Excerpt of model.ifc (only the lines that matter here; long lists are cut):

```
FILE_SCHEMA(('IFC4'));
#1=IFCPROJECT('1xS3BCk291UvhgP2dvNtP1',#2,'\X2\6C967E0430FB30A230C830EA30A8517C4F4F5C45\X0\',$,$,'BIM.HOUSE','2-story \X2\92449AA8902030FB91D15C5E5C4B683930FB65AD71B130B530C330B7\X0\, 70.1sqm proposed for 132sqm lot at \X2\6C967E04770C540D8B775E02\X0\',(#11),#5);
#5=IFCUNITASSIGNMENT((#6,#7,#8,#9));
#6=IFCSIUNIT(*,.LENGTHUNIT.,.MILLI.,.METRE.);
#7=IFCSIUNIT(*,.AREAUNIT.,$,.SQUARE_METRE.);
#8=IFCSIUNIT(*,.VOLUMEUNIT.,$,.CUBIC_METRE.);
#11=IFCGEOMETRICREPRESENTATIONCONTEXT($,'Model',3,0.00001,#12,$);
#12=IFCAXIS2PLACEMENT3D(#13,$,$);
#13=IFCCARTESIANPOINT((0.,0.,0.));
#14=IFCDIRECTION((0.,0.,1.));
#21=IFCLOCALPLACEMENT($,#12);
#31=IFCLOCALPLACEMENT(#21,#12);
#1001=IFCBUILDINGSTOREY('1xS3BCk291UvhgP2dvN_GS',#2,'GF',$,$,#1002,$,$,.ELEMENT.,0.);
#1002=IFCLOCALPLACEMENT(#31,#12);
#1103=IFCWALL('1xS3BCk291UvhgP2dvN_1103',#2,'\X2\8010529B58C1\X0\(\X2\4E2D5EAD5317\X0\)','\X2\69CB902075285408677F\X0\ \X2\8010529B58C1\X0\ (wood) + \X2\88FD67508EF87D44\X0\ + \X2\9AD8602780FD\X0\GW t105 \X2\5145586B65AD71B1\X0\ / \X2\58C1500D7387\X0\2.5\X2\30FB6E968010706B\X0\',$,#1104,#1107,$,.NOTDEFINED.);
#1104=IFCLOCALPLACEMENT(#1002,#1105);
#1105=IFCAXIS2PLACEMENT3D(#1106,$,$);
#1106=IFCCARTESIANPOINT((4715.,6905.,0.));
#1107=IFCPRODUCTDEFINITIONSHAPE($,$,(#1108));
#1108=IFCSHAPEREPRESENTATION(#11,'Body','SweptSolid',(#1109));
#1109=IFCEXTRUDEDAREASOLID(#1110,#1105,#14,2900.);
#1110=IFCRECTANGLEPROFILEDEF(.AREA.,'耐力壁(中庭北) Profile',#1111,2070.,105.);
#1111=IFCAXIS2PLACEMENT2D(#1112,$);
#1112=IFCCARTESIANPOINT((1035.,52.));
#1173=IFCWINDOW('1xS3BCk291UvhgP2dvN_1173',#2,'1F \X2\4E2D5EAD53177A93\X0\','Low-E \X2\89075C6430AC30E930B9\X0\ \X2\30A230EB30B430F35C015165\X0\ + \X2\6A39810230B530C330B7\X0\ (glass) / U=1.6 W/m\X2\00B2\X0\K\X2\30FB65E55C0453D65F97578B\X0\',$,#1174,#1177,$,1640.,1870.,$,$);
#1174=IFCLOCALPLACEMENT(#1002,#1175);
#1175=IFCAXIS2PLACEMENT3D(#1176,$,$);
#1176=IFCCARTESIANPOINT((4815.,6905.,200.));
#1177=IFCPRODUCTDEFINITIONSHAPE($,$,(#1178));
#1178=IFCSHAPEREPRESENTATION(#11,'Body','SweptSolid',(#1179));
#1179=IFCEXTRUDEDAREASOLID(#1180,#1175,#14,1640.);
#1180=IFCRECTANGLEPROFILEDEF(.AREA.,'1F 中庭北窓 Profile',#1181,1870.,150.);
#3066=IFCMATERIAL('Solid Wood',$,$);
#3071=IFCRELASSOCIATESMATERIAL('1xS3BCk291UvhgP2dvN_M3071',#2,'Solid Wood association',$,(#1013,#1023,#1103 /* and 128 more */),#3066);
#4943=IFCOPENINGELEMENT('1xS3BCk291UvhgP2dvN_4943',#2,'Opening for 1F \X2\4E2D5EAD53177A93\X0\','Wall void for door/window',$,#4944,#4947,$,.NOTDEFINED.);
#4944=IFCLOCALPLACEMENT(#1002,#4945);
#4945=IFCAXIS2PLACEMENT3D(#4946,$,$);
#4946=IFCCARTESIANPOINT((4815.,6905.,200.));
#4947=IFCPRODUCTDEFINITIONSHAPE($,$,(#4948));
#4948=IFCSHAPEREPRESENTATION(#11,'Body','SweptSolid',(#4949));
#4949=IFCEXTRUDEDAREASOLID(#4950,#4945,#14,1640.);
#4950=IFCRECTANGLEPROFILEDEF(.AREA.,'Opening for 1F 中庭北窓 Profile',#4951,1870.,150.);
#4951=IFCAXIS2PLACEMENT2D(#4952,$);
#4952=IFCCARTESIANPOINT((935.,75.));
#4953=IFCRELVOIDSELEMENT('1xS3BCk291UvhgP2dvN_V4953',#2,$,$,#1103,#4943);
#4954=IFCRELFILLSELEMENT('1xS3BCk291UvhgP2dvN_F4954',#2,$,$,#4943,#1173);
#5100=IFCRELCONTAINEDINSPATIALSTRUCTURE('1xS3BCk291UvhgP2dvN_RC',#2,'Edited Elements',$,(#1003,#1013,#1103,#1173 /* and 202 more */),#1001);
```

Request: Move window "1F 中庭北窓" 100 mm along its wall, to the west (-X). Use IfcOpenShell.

```python
import ifcopenshell
import ifcopenshell.api.geometry
import ifcopenshell.util.placement

model = ifcopenshell.open("model.ifc")

window = model.by_guid("1xS3BCk291UvhgP2dvN_1173")
opening = window.FillsVoids[0].RelatingOpeningElement
wall = opening.VoidsElements[0].RelatingBuildingElement

wall_matrix = ifcopenshell.util.placement.get_local_placement(wall.ObjectPlacement)
shift = wall_matrix[:3, 0] * -100.0
before = ifcopenshell.util.placement.get_local_placement(window.ObjectPlacement)[:3, 3].copy()

# The window is not placed relative to its opening, so move both.
for product in (opening, window):
    matrix = ifcopenshell.util.placement.get_local_placement(product.ObjectPlacement)
    matrix[:3, 3] += shift
    ifcopenshell.api.geometry.edit_object_placement(model, product=product, matrix=matrix, is_si=False)

after = ifcopenshell.util.placement.get_local_placement(window.ObjectPlacement)[:3, 3]
print("window moved by", (after - before).round(3) + 0.0)

model.write("model_rev.ifc")
```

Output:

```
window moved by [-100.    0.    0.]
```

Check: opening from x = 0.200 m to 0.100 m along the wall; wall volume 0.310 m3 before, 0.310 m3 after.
